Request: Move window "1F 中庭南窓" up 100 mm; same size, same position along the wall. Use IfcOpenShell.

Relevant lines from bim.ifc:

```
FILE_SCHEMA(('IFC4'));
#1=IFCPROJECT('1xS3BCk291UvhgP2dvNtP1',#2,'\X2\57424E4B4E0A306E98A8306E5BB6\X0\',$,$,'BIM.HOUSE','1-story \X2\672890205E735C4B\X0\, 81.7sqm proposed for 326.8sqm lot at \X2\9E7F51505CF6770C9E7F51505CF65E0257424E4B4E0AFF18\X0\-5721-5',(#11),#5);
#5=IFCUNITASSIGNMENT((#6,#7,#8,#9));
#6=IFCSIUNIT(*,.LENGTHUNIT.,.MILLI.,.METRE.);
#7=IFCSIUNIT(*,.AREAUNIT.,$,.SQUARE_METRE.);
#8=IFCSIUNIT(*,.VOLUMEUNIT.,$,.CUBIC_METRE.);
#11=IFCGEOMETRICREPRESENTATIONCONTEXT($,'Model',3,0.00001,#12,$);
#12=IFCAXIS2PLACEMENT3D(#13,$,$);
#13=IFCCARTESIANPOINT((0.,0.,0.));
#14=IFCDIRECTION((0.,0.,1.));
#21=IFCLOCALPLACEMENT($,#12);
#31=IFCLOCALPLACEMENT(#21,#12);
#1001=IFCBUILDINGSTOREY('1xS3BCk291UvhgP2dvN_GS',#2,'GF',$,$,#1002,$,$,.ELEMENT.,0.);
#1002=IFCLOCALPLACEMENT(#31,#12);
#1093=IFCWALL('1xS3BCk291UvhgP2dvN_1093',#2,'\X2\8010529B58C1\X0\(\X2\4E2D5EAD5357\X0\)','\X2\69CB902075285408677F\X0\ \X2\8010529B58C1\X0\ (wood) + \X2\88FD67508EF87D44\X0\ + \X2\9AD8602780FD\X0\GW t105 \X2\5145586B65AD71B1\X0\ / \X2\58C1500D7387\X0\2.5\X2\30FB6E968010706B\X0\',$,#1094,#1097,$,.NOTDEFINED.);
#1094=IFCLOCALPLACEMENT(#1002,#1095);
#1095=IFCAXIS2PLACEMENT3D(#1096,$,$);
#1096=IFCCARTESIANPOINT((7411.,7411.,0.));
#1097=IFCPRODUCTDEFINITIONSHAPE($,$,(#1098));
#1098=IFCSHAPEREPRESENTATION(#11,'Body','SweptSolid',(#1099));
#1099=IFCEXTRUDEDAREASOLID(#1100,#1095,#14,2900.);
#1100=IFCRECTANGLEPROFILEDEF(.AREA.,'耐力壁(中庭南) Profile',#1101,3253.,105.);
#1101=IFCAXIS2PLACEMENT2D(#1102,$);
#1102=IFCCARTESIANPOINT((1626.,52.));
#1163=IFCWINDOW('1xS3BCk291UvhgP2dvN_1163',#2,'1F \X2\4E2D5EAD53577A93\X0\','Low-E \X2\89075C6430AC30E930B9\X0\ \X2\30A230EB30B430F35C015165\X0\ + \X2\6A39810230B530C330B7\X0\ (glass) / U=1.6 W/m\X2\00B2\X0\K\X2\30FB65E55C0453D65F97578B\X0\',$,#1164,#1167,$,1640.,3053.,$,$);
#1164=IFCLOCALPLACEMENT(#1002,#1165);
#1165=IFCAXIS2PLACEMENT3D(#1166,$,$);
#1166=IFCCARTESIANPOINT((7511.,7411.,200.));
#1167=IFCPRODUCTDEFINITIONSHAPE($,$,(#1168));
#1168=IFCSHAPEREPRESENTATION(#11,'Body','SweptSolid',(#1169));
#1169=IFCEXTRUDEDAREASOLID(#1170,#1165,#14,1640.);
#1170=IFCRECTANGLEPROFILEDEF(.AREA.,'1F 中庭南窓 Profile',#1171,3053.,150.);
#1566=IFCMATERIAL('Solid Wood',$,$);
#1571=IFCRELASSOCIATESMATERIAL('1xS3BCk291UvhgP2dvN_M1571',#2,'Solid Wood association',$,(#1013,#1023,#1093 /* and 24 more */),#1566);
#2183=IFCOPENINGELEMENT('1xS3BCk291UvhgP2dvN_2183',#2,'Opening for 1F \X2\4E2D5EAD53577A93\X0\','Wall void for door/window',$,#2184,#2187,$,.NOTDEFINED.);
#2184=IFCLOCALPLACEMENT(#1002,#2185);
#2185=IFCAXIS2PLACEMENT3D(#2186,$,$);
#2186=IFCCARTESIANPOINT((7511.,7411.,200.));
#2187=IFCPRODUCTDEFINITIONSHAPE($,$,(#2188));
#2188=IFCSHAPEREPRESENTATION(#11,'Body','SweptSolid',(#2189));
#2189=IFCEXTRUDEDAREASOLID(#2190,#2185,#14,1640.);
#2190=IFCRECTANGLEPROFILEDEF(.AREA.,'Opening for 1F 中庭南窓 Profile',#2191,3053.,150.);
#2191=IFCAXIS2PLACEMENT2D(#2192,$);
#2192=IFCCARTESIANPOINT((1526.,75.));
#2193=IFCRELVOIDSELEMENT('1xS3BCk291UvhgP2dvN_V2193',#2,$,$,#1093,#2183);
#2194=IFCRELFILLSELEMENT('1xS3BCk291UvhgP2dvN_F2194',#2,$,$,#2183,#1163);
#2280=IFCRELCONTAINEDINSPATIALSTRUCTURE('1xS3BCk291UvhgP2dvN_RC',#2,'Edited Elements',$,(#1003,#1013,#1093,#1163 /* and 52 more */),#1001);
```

```python
import numpy as np
import ifcopenshell
import ifcopenshell.api.geometry
import ifcopenshell.util.placement
import ifcopenshell.util.unit

model = ifcopenshell.open("bim.ifc")
unit_scale = ifcopenshell.util.unit.calculate_unit_scale(model)

window = model.by_id(1163)
opening = window.FillsVoids[0].RelatingOpeningElement
dz = 100.0

shift = np.array([0.0, 0.0, dz])
# The window is not placed relative to its opening, so move both.
for product in (opening, window):
    matrix = ifcopenshell.util.placement.get_local_placement(product.ObjectPlacement)
    matrix[:3, 3] += shift
    ifcopenshell.api.geometry.edit_object_placement(model, product=product, matrix=matrix, is_si=False)

print(f"moved by {dz * unit_scale:+.3f} m")

model.write("bim_v2.ifc")
```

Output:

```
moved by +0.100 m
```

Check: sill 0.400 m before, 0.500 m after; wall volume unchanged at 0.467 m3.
